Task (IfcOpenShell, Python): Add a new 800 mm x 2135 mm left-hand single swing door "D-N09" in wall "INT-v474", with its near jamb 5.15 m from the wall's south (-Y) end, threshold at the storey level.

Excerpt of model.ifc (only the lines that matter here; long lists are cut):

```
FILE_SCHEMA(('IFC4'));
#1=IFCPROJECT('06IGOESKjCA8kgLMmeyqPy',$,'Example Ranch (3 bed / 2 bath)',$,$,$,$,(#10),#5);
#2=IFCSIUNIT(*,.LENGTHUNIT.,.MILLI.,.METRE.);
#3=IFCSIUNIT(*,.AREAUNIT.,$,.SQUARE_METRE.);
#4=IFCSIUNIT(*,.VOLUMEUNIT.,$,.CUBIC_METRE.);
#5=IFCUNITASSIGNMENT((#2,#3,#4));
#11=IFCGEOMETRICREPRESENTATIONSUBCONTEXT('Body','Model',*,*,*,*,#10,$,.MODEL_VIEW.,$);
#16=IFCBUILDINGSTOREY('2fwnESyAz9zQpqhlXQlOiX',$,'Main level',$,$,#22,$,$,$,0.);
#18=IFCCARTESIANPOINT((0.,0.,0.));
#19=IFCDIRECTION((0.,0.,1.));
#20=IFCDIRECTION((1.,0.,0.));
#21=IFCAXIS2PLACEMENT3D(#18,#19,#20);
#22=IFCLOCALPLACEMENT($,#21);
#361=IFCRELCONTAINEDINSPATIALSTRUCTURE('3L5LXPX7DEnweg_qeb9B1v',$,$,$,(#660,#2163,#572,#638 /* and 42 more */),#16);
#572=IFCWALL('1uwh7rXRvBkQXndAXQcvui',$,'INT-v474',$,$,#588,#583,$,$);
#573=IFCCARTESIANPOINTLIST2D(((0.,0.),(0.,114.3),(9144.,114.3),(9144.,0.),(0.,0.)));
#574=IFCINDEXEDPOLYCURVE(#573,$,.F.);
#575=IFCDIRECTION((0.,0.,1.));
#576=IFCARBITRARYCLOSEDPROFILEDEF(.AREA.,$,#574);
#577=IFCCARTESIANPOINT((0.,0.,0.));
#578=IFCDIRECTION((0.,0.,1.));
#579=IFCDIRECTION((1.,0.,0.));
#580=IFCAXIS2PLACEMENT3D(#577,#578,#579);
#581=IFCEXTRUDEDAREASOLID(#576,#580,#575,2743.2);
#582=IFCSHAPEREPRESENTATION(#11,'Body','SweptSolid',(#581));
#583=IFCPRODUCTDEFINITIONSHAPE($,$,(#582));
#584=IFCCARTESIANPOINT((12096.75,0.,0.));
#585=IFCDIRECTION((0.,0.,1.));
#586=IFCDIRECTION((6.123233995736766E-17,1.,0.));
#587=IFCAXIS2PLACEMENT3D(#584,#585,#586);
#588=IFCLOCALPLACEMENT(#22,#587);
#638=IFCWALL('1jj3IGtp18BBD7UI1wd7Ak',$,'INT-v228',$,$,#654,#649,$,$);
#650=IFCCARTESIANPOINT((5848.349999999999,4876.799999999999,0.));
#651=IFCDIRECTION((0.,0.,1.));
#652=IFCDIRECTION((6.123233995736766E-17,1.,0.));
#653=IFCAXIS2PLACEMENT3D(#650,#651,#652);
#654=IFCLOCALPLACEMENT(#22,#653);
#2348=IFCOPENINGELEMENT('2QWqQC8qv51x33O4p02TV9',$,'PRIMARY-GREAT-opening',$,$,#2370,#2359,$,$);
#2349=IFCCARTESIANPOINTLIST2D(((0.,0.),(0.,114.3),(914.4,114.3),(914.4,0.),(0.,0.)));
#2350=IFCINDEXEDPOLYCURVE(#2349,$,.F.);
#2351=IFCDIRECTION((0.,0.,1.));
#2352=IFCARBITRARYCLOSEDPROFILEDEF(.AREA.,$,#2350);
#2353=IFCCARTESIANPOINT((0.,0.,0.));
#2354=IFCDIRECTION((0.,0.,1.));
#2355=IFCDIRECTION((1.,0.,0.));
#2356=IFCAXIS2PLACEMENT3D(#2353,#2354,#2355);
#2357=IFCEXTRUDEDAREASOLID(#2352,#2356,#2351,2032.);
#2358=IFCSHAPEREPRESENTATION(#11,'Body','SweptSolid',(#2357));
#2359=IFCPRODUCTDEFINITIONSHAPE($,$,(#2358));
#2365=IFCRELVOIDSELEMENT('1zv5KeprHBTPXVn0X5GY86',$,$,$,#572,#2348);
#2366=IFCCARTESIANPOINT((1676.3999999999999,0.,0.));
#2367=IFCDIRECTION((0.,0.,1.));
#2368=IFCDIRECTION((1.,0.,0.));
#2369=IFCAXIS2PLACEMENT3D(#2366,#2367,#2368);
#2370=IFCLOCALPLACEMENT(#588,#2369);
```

```python
import numpy as np
import ifcopenshell
import ifcopenshell.api.feature
import ifcopenshell.api.geometry
import ifcopenshell.api.root
import ifcopenshell.api.spatial
import ifcopenshell.geom
import ifcopenshell.util.element
import ifcopenshell.util.placement
import ifcopenshell.util.representation
import ifcopenshell.util.shape
import ifcopenshell.util.unit

model = ifcopenshell.open("model.ifc")
unit_scale = ifcopenshell.util.unit.calculate_unit_scale(model)
settings = ifcopenshell.geom.settings()


def volume(element):
    """Net volume in cubic metres, openings subtracted."""
    shape = ifcopenshell.geom.create_shape(settings, element)
    return ifcopenshell.util.shape.get_volume(shape.geometry)


wall = model.by_id(572)
storey = ifcopenshell.util.element.get_container(wall, ifc_class="IfcBuildingStorey")
context = ifcopenshell.util.representation.get_context(model, "Model", "Body", "MODEL_VIEW")
before = volume(wall)

width, height, from_end, sill = 0.8, 2.135, 5.15, 0.0  # metres

# The wall runs along its own X axis, and the end named is its -X end.
wall_shape = ifcopenshell.geom.create_shape(settings, wall)
x, y, z = ifcopenshell.util.shape.get_vertices(wall_shape.geometry).T
start = x.min() + from_end
face, thickness = float(y.min()), float(y.max() - y.min())
wall_matrix = ifcopenshell.util.placement.get_local_placement(wall.ObjectPlacement)
level = ifcopenshell.util.placement.get_local_placement(storey.ObjectPlacement)[2, 3]


def in_wall(x, y):
    """Placement at x, y metres in the wall's axes, at sill height."""
    matrix = wall_matrix.copy()
    matrix[:, 3] = wall_matrix @ np.array([x / unit_scale, y / unit_scale, 0.0, 1.0])
    matrix[2, 3] = level + sill / unit_scale
    return matrix


# Opening: a box that overshoots both wall faces by 50 mm.
opening = ifcopenshell.api.root.create_entity(model, ifc_class="IfcOpeningElement", predefined_type="OPENING")
box = ifcopenshell.api.geometry.add_wall_representation(
    model, context=context, length=width, height=height, thickness=thickness + 0.1
)
ifcopenshell.api.geometry.assign_representation(model, product=opening, representation=box)
ifcopenshell.api.geometry.edit_object_placement(model, product=opening, matrix=in_wall(start, face - 0.05), is_si=False)
ifcopenshell.api.feature.add_feature(model, feature=opening, element=wall)

door = ifcopenshell.api.root.create_entity(model, ifc_class="IfcDoor", name="D-N09", predefined_type="DOOR")
door.OverallWidth, door.OverallHeight = width / unit_scale, height / unit_scale
door.OperationType = "SINGLE_SWING_LEFT"
body = ifcopenshell.api.geometry.add_door_representation(
    model,
    context=context,
    overall_width=door.OverallWidth,
    overall_height=door.OverallHeight,
    operation_type="SINGLE_SWING_LEFT",
    lining_properties={"LiningDepth": thickness / unit_scale, "ThresholdDepth": thickness / unit_scale},
)
ifcopenshell.api.geometry.assign_representation(model, product=door, representation=body)
ifcopenshell.api.spatial.assign_container(model, products=[door], relating_structure=storey)
ifcopenshell.api.feature.add_filling(model, opening=opening, element=door)

# The lining spans the wall, so the door starts at the wall face.
ifcopenshell.api.geometry.edit_object_placement(model, product=door, matrix=in_wall(start, face), is_si=False)

after = volume(wall)

print(f"wall volume {before:.3f} -> {after:.3f} m3")

model.write("model_rev.ifc")
```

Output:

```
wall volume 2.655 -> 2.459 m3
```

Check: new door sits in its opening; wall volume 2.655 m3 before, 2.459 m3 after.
